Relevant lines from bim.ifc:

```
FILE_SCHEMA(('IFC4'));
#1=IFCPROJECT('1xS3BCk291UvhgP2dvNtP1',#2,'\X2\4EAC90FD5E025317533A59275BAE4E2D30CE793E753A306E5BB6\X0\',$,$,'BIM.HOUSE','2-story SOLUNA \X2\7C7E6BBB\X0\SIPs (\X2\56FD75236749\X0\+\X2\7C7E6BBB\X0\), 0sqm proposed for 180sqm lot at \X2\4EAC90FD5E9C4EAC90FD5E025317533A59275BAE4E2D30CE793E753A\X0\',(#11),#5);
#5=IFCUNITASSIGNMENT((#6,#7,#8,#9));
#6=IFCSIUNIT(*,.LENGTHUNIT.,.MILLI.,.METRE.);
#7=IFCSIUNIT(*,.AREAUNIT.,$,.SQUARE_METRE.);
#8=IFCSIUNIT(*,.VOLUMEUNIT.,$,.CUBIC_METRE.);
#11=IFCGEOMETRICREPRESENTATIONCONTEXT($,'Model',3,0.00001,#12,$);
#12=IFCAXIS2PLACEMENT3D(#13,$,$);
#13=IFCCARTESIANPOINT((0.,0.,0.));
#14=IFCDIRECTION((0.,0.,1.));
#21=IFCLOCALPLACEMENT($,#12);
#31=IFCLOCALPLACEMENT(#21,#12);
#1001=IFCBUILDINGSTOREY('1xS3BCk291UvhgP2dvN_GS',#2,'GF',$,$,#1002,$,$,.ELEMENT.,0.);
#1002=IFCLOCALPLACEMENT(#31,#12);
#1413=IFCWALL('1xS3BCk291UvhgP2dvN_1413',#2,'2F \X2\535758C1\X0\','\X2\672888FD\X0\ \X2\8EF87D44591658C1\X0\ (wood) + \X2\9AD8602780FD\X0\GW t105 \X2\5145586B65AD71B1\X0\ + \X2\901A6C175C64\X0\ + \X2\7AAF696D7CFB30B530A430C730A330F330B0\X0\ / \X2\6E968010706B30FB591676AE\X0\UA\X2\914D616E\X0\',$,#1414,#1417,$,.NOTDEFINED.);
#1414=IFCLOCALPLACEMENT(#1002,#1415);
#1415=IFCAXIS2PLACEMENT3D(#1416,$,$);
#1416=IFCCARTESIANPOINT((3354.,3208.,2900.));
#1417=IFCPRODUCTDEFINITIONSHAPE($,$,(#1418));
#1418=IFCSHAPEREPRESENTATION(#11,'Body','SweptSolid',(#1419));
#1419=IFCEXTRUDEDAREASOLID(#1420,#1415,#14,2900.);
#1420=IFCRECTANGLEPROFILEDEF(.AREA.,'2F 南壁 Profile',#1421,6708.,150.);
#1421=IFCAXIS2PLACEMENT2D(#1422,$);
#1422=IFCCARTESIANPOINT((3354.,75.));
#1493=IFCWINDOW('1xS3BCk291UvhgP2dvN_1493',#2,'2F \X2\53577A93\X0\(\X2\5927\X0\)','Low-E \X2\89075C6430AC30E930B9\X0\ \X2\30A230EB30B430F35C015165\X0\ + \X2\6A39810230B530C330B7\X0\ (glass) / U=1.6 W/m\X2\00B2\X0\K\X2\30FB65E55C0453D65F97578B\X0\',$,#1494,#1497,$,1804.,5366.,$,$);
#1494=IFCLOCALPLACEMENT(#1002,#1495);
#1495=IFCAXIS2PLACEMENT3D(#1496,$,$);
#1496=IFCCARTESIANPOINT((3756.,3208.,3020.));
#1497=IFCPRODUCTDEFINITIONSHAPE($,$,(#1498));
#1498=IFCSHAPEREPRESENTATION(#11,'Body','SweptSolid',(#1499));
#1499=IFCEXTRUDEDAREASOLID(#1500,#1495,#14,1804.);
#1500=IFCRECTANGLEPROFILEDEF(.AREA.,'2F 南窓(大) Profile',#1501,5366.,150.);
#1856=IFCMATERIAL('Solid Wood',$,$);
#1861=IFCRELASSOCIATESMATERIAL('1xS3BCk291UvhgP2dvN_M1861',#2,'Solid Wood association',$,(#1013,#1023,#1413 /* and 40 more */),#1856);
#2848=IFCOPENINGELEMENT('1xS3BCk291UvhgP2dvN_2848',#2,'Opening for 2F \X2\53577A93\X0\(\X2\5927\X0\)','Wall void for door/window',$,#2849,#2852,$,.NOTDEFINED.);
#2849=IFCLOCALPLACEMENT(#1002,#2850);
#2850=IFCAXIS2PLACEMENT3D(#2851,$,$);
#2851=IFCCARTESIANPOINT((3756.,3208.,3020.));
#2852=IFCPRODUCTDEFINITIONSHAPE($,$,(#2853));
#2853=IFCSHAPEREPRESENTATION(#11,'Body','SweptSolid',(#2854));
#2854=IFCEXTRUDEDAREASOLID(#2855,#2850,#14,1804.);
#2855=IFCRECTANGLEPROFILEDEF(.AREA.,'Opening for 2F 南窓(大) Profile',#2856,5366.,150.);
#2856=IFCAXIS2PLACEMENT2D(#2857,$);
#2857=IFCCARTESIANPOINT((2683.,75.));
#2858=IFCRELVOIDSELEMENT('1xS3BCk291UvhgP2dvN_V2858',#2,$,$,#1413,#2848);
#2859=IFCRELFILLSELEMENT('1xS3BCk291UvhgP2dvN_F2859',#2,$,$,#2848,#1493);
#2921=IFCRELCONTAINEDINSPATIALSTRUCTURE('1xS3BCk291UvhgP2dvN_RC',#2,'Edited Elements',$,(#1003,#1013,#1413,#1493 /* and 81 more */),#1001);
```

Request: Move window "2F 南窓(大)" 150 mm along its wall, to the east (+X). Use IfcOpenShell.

```python
import ifcopenshell
import ifcopenshell.api.geometry
import ifcopenshell.util.placement
import ifcopenshell.util.unit

model = ifcopenshell.open("bim.ifc")
unit_scale = ifcopenshell.util.unit.calculate_unit_scale(model)

window = model.by_id(1493)
opening = window.FillsVoids[0].RelatingOpeningElement
wall = opening.VoidsElements[0].RelatingBuildingElement

wall_matrix = ifcopenshell.util.placement.get_local_placement(wall.ObjectPlacement)
shift = wall_matrix[:3, 0] * 0.15 / unit_scale
before = ifcopenshell.util.placement.get_local_placement(window.ObjectPlacement)[:3, 3].copy()

# The window is not placed relative to its opening, so move both.
for product in (opening, window):
    matrix = ifcopenshell.util.placement.get_local_placement(product.ObjectPlacement)
    matrix[:3, 3] += shift
    ifcopenshell.api.geometry.edit_object_placement(model, product=product, matrix=matrix, is_si=False)

after = ifcopenshell.util.placement.get_local_placement(window.ObjectPlacement)[:3, 3]
print("window moved by", (after - before).round(3) + 0.0)

model.write("bim_edited.ifc")
```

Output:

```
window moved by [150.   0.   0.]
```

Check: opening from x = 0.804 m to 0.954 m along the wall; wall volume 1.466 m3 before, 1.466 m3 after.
